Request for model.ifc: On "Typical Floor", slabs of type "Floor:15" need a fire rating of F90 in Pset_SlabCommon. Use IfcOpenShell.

First a look at what the model holds.

```python
import ifcopenshell
import ifcopenshell.util.element

model = ifcopenshell.open("model.ifc")
print(model.schema)
storey = next(s for s in model.by_type("IfcBuildingStorey") if s.Name == "Typical Floor")
slabs = [e for e in ifcopenshell.util.element.get_decomposition(storey) if e.is_a("IfcSlab")]
seen = {}
for e in slabs:
    element_type = ifcopenshell.util.element.get_type(e)
    key = (element_type.Name if element_type != e and element_type else None, ifcopenshell.util.element.get_pset(e, "Pset_SlabCommon", "FireRating"))
    seen[key] = seen.get(key, 0) + 1
for (name, value), count in sorted(seen.items(), key=str):
    print(count, "x", name, "|", value)
```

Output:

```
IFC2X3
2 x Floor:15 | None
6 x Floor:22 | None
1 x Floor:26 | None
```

```python
import ifcopenshell
import ifcopenshell.api.pset
import ifcopenshell.util.element

model = ifcopenshell.open("model.ifc")

storey = next(s for s in model.by_type("IfcBuildingStorey") if s.Name == "Typical Floor")
slabs = [e for e in ifcopenshell.util.element.get_decomposition(storey) if e.is_a("IfcSlab")]

count = 0
for e in slabs:
    element_type = ifcopenshell.util.element.get_type(e)
    if element_type in (None, e) or element_type.Name != "Floor:15":
        continue
    # add_pset returns the element's existing set when there is one.
    pset = ifcopenshell.api.pset.add_pset(model, product=e, name="Pset_SlabCommon")
    ifcopenshell.api.pset.edit_pset(model, pset=pset, properties={"FireRating": "F90"})
    count += 1

print(count, "slabs updated")

model.write("model_updated.ifc")
```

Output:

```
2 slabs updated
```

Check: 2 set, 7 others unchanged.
